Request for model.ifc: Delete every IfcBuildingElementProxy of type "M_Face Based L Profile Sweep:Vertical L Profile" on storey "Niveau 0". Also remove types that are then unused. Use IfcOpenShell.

First a look at what the model holds.

```python
import ifcopenshell
import ifcopenshell.util.element

model = ifcopenshell.open("model.ifc")
print(model.schema)
storey = next(s for s in model.by_type("IfcBuildingStorey") if s.Name == "Niveau 0")
proxies = [e for e in ifcopenshell.util.element.get_decomposition(storey) if e.is_a("IfcBuildingElementProxy")]
seen = {}
for e in proxies:
    element_type = ifcopenshell.util.element.get_type(e)
    name = element_type.Name if element_type not in (None, e) else None
    seen[name] = seen.get(name, 0) + 1
for name, count in sorted(seen.items(), key=str):
    print(count, "x", name)
```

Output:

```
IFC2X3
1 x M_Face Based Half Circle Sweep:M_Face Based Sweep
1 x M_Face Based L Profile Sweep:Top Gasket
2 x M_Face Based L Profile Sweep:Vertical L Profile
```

```python
import ifcopenshell
import ifcopenshell.api.root
import ifcopenshell.util.element

model = ifcopenshell.open("model.ifc")

storey = next(s for s in model.by_type("IfcBuildingStorey") if s.Name == "Niveau 0")
proxies = [e for e in ifcopenshell.util.element.get_decomposition(storey) if e.is_a("IfcBuildingElementProxy")]
targets = [e for e in proxies if (t := ifcopenshell.util.element.get_type(e)) not in (None, e) and t.Name == "M_Face Based L Profile Sweep:Vertical L Profile"]
types = {ifcopenshell.util.element.get_type(e) for e in targets} - {None, *targets}

for e in targets:
    ifcopenshell.api.root.remove_product(model, product=e)
print(len(targets), "removed")

unused = [t for t in types if not ifcopenshell.util.element.get_types(t)]
for t in unused:
    ifcopenshell.api.root.remove_product(model, product=t)
print(len(unused), "unused types removed")

model.write("model-out.ifc")
```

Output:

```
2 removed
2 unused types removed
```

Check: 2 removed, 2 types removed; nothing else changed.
